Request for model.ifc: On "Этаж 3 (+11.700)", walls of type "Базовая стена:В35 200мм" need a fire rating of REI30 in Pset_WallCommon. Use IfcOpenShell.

First a look at what the model holds.

```python
import ifcopenshell
import ifcopenshell.util.element

model = ifcopenshell.open("model.ifc")
print(model.schema)
storey = next(s for s in model.by_type("IfcBuildingStorey") if s.Name == "Этаж 3 (+11.700)")
walls = [e for e in ifcopenshell.util.element.get_decomposition(storey) if e.is_a("IfcWall")]
seen = {}
for e in walls:
    element_type = ifcopenshell.util.element.get_type(e)
    key = (element_type.Name if element_type != e and element_type else None, ifcopenshell.util.element.get_pset(e, "Pset_WallCommon", "FireRating"))
    seen[key] = seen.get(key, 0) + 1
for (name, value), count in sorted(seen.items(), key=str):
    print(count, "x", name, "|", value)
```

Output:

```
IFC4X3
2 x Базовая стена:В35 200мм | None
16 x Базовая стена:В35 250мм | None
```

```python
import ifcopenshell
import ifcopenshell.api.pset
import ifcopenshell.util.element

model = ifcopenshell.open("model.ifc")

storey = next(s for s in model.by_type("IfcBuildingStorey") if s.Name == "Этаж 3 (+11.700)")
walls = [e for e in ifcopenshell.util.element.get_decomposition(storey) if e.is_a("IfcWall")]

count = 0
for e in walls:
    element_type = ifcopenshell.util.element.get_type(e)
    if element_type in (None, e) or element_type.Name != "Базовая стена:В35 200мм":
        continue
    # add_pset returns the element's existing set when there is one.
    pset = ifcopenshell.api.pset.add_pset(model, product=e, name="Pset_WallCommon")
    ifcopenshell.api.pset.edit_pset(model, pset=pset, properties={"FireRating": "REI30"})
    count += 1

print(count, "walls updated")

model.write("model_v2.ifc")
```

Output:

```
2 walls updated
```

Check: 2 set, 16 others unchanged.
